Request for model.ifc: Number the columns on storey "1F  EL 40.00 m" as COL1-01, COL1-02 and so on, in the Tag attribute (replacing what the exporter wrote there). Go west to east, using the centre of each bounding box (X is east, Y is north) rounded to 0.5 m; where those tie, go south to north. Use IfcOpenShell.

First a look at what the model holds.

```python
import ifcopenshell
import ifcopenshell.util.element
import ifcopenshell.util.placement

model = ifcopenshell.open("model.ifc")
print(model.schema)
storey = next(s for s in model.by_type("IfcBuildingStorey") if s.Name == "1F  EL 40.00 m")
columns = [e for e in ifcopenshell.util.element.get_decomposition(storey) if e.is_a("IfcColumn")]
for e in sorted(columns, key=lambda e: e.id()):
    origin = ifcopenshell.util.placement.get_local_placement(e.ObjectPlacement)[:3, 3]
    print(e.id(), e.Tag, e.Name, origin.round(2) + 0.0, sep=" | ")
```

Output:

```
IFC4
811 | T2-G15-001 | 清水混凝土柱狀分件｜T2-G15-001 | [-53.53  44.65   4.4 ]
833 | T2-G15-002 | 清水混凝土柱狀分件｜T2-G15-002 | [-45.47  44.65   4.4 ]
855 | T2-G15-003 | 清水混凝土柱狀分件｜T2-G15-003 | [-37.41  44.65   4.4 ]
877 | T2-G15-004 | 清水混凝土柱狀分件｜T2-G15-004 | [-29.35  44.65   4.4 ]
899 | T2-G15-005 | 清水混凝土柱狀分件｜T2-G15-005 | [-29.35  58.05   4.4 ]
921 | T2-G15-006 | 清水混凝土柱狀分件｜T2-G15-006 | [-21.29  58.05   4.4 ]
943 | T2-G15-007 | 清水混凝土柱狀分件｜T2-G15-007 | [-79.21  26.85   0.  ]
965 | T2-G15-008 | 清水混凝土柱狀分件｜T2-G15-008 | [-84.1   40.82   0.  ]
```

```python
import ifcopenshell
import ifcopenshell.geom
import ifcopenshell.util.element
import ifcopenshell.util.shape

model = ifcopenshell.open("model.ifc")
settings = ifcopenshell.geom.settings()
settings.set("use-world-coords", True)


def centre(element):
    shape = ifcopenshell.geom.create_shape(settings, element)
    return ifcopenshell.util.shape.get_bbox_centroid(shape.geometry)


storey = next(s for s in model.by_type("IfcBuildingStorey") if s.Name == "1F  EL 40.00 m")
columns = [e for e in ifcopenshell.util.element.get_decomposition(storey) if e.is_a("IfcColumn")]

# Insertion points can sit at a corner or the storey origin, so sort by the geometry (in metres).
centres = {e: centre(e) for e in columns}
columns.sort(key=lambda e: (round(centres[e][0] / 0.5), centres[e][1]))

for i, e in enumerate(columns, start=1):
    number = f"COL1-{i:02d}"
    e.Tag = number
    print(e.id(), number)

model.write("model-out.ifc")
```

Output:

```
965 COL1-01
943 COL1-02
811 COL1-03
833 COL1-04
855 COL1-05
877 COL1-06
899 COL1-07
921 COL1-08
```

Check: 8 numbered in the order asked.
